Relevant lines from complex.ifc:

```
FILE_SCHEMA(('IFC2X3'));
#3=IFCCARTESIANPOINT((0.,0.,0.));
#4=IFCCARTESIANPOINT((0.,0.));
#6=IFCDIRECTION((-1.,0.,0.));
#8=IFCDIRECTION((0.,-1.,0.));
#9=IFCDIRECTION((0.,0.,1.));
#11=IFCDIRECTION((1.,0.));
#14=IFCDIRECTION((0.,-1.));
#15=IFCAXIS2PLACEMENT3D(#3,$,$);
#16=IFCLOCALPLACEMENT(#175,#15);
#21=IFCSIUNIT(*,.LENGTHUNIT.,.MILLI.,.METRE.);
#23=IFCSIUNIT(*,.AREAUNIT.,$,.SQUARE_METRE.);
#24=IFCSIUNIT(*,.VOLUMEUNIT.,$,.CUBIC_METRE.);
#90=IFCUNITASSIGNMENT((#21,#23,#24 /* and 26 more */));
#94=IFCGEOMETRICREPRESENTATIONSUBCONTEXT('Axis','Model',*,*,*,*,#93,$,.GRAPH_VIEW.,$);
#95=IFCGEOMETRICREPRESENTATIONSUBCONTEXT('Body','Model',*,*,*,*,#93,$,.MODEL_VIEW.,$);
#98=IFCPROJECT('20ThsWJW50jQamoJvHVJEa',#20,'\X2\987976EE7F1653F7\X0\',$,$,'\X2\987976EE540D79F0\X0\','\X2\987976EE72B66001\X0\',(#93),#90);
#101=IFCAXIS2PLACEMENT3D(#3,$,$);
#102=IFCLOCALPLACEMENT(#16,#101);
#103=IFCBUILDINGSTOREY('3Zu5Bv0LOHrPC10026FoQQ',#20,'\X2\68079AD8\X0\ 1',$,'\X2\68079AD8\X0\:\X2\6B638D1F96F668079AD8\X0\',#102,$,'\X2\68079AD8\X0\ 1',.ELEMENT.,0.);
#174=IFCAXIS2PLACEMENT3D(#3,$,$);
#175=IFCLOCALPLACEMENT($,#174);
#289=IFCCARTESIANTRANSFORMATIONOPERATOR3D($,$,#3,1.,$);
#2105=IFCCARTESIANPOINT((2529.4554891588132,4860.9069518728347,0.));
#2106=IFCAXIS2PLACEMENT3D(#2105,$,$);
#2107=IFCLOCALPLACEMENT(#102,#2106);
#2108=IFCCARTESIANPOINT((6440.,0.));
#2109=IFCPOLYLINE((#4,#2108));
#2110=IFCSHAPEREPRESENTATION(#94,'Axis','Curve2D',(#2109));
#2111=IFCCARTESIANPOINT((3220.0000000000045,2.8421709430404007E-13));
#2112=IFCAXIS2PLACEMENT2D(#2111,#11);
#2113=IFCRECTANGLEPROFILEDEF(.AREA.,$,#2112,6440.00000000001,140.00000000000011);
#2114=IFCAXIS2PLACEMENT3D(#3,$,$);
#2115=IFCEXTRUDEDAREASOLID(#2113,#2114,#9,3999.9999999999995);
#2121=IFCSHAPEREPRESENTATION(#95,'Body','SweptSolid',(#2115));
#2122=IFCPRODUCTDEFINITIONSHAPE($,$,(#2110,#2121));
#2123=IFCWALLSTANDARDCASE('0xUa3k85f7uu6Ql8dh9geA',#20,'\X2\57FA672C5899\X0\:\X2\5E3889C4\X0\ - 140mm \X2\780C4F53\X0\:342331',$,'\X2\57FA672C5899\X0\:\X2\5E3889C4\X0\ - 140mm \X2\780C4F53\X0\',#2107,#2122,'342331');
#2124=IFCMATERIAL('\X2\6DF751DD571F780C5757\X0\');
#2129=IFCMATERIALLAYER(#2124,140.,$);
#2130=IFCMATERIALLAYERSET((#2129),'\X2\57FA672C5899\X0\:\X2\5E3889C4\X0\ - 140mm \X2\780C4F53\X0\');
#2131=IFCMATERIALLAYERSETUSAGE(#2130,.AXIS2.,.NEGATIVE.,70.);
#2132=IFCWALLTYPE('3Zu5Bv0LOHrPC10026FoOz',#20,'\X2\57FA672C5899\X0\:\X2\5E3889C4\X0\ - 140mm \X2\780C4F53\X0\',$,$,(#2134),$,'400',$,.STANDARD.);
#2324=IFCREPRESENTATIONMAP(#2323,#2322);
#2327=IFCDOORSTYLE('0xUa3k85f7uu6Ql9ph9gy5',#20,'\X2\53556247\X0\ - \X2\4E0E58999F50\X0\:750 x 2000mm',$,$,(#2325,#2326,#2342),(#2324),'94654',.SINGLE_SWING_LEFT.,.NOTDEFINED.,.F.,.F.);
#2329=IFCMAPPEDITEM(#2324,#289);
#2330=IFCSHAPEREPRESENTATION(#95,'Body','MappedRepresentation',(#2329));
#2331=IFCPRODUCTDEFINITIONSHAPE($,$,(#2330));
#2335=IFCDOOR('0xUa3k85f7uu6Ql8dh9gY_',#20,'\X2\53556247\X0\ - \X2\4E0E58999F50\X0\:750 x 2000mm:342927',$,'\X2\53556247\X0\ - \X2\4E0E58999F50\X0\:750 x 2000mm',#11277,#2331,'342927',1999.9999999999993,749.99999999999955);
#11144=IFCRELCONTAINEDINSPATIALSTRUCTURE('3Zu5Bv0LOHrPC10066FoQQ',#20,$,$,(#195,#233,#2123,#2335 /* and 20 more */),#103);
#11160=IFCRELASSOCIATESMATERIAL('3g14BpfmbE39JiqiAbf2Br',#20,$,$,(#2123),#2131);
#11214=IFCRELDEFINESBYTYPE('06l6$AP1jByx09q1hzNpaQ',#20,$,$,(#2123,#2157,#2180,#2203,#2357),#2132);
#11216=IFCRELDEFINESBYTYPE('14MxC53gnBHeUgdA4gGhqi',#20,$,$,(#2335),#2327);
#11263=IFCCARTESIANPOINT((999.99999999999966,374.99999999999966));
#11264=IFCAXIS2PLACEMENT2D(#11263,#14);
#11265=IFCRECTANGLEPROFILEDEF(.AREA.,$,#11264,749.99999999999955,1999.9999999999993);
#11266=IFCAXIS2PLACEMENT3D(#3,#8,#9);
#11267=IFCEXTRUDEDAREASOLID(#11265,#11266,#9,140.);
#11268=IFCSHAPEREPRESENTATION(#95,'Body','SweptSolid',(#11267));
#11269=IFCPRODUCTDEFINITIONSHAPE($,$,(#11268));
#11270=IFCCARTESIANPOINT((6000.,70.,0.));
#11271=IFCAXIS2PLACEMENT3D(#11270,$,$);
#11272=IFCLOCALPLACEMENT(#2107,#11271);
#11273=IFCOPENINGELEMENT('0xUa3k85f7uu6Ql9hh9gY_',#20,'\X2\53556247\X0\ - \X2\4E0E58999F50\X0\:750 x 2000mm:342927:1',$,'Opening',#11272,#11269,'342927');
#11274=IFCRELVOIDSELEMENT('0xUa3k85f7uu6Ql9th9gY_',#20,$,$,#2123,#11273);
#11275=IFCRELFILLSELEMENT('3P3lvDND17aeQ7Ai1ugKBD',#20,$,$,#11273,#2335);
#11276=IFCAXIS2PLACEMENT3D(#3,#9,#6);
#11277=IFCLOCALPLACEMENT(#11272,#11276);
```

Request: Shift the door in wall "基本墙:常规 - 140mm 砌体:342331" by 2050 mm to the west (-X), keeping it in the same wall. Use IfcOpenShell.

```python
import ifcopenshell
import ifcopenshell.api.geometry
import ifcopenshell.util.placement
import ifcopenshell.util.unit

model = ifcopenshell.open("complex.ifc")
unit_scale = ifcopenshell.util.unit.calculate_unit_scale(model)

door = model.by_id(2335)
opening = door.FillsVoids[0].RelatingOpeningElement
wall = opening.VoidsElements[0].RelatingBuildingElement

wall_matrix = ifcopenshell.util.placement.get_local_placement(wall.ObjectPlacement)
shift = wall_matrix[:3, 0] * -2.05 / unit_scale
before = ifcopenshell.util.placement.get_local_placement(door.ObjectPlacement)[:3, 3].copy()

# The door is placed relative to its opening, so it follows when the opening moves.
matrix = ifcopenshell.util.placement.get_local_placement(opening.ObjectPlacement)
matrix[:3, 3] += shift
ifcopenshell.api.geometry.edit_object_placement(
    model, product=opening, matrix=matrix, is_si=False, should_transform_children=True
)

after = ifcopenshell.util.placement.get_local_placement(door.ObjectPlacement)[:3, 3]
print("door moved by", (after - before).round(3) + 0.0)

model.write("complex_v2.ifc")
```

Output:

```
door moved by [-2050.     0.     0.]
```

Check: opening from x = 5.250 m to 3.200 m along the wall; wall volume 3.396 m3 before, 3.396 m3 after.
